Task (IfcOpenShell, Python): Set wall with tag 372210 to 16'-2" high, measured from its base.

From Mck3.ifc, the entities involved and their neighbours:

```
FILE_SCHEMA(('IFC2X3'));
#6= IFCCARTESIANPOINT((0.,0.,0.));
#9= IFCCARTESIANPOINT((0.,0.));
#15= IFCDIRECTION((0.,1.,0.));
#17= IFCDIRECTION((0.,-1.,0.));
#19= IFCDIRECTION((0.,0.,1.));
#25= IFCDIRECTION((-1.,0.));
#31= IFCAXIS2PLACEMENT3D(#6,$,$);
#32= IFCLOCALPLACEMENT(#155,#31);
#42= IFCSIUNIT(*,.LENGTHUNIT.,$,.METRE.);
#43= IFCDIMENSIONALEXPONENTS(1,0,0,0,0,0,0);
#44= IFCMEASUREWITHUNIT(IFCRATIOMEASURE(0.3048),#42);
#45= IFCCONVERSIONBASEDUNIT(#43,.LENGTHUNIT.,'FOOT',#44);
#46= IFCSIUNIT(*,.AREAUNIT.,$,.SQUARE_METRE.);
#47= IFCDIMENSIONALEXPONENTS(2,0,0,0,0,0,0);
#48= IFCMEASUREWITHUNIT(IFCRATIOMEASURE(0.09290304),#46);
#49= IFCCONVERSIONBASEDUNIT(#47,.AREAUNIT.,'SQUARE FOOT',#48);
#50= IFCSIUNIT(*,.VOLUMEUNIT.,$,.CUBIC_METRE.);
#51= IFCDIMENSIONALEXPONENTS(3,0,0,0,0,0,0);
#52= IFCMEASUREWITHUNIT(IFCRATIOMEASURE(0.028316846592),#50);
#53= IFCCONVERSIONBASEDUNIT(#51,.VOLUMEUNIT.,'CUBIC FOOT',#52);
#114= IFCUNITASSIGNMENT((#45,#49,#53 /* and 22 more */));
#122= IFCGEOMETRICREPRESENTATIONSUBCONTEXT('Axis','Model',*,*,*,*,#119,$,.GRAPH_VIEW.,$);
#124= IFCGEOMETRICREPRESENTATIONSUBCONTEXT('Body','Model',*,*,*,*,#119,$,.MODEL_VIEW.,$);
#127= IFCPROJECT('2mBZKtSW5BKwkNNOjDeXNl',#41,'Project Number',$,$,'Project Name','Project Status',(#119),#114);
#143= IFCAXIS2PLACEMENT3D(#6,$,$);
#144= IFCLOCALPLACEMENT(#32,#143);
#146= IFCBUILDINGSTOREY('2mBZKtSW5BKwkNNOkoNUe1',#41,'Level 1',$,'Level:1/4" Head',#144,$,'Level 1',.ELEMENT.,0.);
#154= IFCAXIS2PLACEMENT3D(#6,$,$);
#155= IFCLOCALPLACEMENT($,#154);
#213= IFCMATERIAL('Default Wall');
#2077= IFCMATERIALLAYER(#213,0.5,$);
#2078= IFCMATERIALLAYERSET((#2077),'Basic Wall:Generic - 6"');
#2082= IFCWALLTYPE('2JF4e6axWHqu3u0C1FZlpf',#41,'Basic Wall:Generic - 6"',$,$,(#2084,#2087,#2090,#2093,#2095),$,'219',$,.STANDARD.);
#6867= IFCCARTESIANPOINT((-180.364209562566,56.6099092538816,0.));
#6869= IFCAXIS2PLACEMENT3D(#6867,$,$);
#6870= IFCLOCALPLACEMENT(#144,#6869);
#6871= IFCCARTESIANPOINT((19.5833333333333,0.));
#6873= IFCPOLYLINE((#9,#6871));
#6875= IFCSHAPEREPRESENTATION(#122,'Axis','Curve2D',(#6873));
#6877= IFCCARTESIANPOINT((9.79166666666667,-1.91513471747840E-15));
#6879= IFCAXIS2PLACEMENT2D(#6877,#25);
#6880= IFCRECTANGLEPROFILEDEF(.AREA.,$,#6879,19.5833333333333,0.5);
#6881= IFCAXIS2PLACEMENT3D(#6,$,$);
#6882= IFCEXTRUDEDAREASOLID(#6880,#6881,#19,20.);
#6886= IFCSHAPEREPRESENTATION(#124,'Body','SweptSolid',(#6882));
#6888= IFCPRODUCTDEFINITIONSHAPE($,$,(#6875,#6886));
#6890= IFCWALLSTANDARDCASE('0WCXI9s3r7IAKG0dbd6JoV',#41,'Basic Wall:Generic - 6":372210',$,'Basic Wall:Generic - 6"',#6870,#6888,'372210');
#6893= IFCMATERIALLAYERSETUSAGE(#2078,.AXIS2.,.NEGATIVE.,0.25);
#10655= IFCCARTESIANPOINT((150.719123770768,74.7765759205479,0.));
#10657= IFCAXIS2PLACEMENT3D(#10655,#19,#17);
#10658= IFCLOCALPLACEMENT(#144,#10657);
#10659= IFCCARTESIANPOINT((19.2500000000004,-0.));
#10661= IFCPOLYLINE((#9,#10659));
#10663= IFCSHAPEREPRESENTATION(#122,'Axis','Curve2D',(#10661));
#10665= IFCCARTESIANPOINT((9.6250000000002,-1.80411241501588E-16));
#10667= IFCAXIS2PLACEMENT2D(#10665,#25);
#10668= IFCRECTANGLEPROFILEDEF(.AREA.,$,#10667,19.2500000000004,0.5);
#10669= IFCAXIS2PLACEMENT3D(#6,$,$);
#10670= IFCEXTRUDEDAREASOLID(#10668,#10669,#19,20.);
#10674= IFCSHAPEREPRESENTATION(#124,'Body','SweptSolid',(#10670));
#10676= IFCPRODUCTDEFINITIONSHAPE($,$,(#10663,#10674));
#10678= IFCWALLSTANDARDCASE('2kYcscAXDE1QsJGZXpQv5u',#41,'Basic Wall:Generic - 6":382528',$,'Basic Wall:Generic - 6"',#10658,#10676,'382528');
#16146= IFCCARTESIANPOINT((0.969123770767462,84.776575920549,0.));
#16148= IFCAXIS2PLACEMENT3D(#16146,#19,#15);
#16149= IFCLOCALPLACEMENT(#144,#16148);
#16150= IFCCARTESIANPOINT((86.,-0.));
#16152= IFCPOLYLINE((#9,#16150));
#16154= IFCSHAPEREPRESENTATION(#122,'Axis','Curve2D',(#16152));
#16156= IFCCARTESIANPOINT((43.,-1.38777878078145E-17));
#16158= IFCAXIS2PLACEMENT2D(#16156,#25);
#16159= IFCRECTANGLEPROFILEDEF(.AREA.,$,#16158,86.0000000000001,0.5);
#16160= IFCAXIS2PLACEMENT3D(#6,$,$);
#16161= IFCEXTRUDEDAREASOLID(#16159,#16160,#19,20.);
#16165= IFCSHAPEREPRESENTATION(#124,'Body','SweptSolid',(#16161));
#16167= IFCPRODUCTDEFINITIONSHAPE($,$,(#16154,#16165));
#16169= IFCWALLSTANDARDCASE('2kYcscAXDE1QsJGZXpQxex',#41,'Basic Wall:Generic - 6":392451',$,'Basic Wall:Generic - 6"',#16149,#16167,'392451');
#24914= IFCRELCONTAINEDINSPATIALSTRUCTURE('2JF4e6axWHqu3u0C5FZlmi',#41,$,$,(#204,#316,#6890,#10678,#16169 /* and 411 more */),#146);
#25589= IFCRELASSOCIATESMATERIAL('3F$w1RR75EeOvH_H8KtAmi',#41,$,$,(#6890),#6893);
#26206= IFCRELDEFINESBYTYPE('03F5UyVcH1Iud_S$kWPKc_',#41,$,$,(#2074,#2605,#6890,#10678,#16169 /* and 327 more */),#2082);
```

```python
import ifcopenshell
import ifcopenshell.geom
import ifcopenshell.util.representation
import ifcopenshell.util.shape
import ifcopenshell.util.unit

model = ifcopenshell.open("Mck3.ifc")
unit_scale = ifcopenshell.util.unit.calculate_unit_scale(model)
settings = ifcopenshell.geom.settings()


def volume(element):
    """Net volume in cubic metres, openings subtracted."""
    shape = ifcopenshell.geom.create_shape(settings, element)
    return ifcopenshell.util.shape.get_volume(shape.geometry)


wall = model.by_guid("0WCXI9s3r7IAKG0dbd6JoV")
before = volume(wall)

body = ifcopenshell.util.representation.get_representation(wall, "Model", "Body")
solid = body.Items[0]
old_height = solid.Depth
solid.Depth = 194 * 0.0254 / unit_scale
after = volume(wall)

print(f"height {old_height:g} -> {solid.Depth:g}, volume {before:.3f} -> {after:.3f} m3")

model.write("Mck3-out.ifc")
```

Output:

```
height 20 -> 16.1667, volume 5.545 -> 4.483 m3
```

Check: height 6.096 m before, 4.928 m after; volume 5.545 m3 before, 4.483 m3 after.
